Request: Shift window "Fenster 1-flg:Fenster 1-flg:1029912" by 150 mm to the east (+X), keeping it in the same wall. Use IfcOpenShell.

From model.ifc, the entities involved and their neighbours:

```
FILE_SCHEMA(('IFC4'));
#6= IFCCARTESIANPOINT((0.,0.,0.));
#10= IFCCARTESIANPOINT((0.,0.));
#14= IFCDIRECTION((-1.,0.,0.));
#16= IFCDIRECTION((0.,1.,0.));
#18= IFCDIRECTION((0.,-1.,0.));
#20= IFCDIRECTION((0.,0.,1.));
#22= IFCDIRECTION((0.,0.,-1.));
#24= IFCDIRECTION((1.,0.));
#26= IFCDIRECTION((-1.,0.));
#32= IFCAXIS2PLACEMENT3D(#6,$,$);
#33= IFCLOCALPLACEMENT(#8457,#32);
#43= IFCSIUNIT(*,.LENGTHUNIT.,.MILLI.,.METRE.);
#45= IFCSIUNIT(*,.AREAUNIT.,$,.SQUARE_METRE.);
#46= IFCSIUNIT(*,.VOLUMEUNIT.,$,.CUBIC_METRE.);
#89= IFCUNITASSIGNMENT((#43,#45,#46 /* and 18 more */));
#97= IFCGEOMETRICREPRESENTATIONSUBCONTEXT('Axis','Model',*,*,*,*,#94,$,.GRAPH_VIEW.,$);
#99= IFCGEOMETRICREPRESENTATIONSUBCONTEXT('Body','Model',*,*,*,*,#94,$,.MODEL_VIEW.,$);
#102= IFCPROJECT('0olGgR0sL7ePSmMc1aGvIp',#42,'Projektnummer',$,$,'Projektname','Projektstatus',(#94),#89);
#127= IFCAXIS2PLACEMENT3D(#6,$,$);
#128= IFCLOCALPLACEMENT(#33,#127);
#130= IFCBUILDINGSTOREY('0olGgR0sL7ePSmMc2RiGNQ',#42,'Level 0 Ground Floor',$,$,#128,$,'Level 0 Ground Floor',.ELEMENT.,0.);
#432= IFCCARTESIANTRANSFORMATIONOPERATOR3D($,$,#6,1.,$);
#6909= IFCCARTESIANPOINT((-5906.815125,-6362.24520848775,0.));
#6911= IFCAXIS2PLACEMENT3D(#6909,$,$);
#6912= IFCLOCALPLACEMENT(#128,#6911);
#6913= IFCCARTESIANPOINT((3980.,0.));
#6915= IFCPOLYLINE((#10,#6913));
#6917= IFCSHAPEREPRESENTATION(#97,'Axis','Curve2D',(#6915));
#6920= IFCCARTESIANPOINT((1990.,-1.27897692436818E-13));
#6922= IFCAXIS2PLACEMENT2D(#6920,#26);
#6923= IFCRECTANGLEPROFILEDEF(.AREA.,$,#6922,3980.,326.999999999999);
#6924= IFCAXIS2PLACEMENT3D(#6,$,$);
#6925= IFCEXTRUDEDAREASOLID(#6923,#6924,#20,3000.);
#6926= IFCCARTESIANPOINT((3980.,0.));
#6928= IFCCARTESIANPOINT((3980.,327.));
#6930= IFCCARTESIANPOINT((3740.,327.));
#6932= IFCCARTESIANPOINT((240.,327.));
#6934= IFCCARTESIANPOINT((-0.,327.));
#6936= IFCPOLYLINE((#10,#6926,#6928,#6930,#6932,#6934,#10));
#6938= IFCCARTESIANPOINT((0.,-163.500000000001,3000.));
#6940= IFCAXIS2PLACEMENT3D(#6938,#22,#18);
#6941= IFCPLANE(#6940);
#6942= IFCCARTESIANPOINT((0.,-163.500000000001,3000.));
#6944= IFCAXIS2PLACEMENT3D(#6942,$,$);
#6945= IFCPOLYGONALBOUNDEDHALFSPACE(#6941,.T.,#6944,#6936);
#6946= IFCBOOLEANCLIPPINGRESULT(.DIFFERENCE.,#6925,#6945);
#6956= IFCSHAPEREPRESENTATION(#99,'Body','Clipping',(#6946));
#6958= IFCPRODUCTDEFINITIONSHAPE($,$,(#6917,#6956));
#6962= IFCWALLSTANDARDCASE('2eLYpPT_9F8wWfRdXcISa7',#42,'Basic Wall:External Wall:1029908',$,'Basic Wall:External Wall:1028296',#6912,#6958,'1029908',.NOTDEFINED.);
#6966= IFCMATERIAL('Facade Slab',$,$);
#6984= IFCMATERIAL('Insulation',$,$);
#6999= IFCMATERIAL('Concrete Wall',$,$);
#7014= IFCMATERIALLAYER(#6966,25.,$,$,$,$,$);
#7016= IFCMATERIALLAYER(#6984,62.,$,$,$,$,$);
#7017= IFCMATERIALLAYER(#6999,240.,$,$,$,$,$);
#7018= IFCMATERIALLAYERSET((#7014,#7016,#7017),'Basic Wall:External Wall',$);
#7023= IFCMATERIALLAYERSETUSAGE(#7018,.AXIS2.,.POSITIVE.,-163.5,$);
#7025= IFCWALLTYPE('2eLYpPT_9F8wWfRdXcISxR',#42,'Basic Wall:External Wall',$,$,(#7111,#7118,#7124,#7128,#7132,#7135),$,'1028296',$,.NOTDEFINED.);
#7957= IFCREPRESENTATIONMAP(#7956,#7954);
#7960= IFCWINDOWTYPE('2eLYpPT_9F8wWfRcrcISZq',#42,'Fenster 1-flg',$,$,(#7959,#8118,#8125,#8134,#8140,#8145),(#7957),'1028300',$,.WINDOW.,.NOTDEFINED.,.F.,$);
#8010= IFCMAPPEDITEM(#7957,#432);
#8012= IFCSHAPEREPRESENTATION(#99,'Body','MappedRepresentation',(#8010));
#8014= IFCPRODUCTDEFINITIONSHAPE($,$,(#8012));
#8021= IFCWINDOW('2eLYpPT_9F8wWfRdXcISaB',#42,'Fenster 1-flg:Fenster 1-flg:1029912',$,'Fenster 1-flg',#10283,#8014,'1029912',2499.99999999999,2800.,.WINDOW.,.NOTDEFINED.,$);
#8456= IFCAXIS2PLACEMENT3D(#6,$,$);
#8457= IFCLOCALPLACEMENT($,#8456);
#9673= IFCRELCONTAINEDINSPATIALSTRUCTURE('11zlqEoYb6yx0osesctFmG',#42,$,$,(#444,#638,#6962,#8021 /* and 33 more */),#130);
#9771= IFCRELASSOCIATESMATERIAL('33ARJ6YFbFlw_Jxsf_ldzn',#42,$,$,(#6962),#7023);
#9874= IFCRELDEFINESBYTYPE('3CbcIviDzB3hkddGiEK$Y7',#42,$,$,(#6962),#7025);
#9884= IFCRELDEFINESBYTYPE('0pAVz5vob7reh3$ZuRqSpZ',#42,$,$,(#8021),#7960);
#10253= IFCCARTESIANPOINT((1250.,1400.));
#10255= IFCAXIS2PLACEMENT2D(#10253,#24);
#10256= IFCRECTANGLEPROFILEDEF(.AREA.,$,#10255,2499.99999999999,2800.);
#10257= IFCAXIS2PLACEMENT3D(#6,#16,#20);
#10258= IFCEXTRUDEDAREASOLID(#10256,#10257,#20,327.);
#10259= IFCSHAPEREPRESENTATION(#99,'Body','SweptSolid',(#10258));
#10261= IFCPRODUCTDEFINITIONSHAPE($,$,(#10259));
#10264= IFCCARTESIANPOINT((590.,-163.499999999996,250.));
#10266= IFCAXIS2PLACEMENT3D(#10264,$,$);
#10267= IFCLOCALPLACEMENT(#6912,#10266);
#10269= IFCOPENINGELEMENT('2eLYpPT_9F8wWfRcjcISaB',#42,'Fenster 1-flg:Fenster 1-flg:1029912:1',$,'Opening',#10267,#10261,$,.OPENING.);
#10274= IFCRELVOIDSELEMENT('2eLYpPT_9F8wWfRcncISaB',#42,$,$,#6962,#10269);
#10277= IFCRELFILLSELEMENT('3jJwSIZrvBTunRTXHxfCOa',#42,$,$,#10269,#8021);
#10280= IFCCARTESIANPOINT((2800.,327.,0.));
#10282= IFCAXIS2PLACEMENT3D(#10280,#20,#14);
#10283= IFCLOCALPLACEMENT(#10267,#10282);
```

```python
import ifcopenshell
import ifcopenshell.api.geometry
import ifcopenshell.util.placement
import ifcopenshell.util.unit

model = ifcopenshell.open("model.ifc")
unit_scale = ifcopenshell.util.unit.calculate_unit_scale(model)

window = model.by_guid("2eLYpPT_9F8wWfRdXcISaB")
opening = window.FillsVoids[0].RelatingOpeningElement
wall = opening.VoidsElements[0].RelatingBuildingElement

wall_matrix = ifcopenshell.util.placement.get_local_placement(wall.ObjectPlacement)
shift = wall_matrix[:3, 0] * 0.15 / unit_scale
before = ifcopenshell.util.placement.get_local_placement(window.ObjectPlacement)[:3, 3].copy()

# The window is placed relative to its opening, so it follows when the opening moves.
matrix = ifcopenshell.util.placement.get_local_placement(opening.ObjectPlacement)
matrix[:3, 3] += shift
ifcopenshell.api.geometry.edit_object_placement(
    model, product=opening, matrix=matrix, is_si=False, should_transform_children=True
)

after = ifcopenshell.util.placement.get_local_placement(window.ObjectPlacement)[:3, 3]
print("window moved by", (after - before).round(3) + 0.0)

model.write("model_v2.ifc")
```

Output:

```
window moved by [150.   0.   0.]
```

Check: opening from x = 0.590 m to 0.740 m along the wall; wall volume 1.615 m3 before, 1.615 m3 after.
